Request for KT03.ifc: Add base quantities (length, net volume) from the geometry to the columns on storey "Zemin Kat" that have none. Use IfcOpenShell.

First a look at what the model holds.

```python
import ifcopenshell
import ifcopenshell.util.element
import ifcopenshell.util.unit

model = ifcopenshell.open("KT03.ifc")
print(model.schema)
for unit_type in ("LENGTHUNIT", "AREAUNIT", "VOLUMEUNIT"):
    print(unit_type, ifcopenshell.util.unit.calculate_unit_scale(model, unit_type))
storey = next(s for s in model.by_type("IfcBuildingStorey") if s.Name == "Zemin Kat")
columns = [e for e in ifcopenshell.util.element.get_decomposition(storey) if e.is_a("IfcColumn")]
for e in sorted(columns, key=lambda e: e.id()):
    print(e.id(), e.is_a(), e.Name, list(ifcopenshell.util.element.get_psets(e, qtos_only=True)), sep=" | ")
```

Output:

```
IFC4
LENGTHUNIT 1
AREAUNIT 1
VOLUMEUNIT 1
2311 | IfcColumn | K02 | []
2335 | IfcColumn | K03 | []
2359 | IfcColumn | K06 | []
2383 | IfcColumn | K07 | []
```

```python
import ifcopenshell
import ifcopenshell.api.pset
import ifcopenshell.geom
import ifcopenshell.util.element
import ifcopenshell.util.shape
import ifcopenshell.util.unit

model = ifcopenshell.open("KT03.ifc")
unit_scale = ifcopenshell.util.unit.calculate_unit_scale(model)
volume_scale = ifcopenshell.util.unit.calculate_unit_scale(model, "VOLUMEUNIT")
settings = ifcopenshell.geom.settings()

storey = next(s for s in model.by_type("IfcBuildingStorey") if s.Name == "Zemin Kat")
columns = [e for e in ifcopenshell.util.element.get_decomposition(storey) if e.is_a("IfcColumn")]

for e in sorted(columns, key=lambda e: e.id()):
    if ifcopenshell.util.element.get_psets(e, qtos_only=True, should_inherit=False):
        continue
    # Geometry comes back in metres, in the element's own axes.
    shape = ifcopenshell.geom.create_shape(settings, e)
    values = {
        "Length": ifcopenshell.util.shape.get_z(shape.geometry) / unit_scale,
        "NetVolume": ifcopenshell.util.shape.get_volume(shape.geometry) / volume_scale,
    }
    qto = ifcopenshell.api.pset.add_qto(model, product=e, name="Qto_ColumnBaseQuantities")
    ifcopenshell.api.pset.edit_qto(model, qto=qto, properties=values)
    print(e.id(), {k: round(v, 3) for k, v in values.items()})

model.write("KT03_rev.ifc")
```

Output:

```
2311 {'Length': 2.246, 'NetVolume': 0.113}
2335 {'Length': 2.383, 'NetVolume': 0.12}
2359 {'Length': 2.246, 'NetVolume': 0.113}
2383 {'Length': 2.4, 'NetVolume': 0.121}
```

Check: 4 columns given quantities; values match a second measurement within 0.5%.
